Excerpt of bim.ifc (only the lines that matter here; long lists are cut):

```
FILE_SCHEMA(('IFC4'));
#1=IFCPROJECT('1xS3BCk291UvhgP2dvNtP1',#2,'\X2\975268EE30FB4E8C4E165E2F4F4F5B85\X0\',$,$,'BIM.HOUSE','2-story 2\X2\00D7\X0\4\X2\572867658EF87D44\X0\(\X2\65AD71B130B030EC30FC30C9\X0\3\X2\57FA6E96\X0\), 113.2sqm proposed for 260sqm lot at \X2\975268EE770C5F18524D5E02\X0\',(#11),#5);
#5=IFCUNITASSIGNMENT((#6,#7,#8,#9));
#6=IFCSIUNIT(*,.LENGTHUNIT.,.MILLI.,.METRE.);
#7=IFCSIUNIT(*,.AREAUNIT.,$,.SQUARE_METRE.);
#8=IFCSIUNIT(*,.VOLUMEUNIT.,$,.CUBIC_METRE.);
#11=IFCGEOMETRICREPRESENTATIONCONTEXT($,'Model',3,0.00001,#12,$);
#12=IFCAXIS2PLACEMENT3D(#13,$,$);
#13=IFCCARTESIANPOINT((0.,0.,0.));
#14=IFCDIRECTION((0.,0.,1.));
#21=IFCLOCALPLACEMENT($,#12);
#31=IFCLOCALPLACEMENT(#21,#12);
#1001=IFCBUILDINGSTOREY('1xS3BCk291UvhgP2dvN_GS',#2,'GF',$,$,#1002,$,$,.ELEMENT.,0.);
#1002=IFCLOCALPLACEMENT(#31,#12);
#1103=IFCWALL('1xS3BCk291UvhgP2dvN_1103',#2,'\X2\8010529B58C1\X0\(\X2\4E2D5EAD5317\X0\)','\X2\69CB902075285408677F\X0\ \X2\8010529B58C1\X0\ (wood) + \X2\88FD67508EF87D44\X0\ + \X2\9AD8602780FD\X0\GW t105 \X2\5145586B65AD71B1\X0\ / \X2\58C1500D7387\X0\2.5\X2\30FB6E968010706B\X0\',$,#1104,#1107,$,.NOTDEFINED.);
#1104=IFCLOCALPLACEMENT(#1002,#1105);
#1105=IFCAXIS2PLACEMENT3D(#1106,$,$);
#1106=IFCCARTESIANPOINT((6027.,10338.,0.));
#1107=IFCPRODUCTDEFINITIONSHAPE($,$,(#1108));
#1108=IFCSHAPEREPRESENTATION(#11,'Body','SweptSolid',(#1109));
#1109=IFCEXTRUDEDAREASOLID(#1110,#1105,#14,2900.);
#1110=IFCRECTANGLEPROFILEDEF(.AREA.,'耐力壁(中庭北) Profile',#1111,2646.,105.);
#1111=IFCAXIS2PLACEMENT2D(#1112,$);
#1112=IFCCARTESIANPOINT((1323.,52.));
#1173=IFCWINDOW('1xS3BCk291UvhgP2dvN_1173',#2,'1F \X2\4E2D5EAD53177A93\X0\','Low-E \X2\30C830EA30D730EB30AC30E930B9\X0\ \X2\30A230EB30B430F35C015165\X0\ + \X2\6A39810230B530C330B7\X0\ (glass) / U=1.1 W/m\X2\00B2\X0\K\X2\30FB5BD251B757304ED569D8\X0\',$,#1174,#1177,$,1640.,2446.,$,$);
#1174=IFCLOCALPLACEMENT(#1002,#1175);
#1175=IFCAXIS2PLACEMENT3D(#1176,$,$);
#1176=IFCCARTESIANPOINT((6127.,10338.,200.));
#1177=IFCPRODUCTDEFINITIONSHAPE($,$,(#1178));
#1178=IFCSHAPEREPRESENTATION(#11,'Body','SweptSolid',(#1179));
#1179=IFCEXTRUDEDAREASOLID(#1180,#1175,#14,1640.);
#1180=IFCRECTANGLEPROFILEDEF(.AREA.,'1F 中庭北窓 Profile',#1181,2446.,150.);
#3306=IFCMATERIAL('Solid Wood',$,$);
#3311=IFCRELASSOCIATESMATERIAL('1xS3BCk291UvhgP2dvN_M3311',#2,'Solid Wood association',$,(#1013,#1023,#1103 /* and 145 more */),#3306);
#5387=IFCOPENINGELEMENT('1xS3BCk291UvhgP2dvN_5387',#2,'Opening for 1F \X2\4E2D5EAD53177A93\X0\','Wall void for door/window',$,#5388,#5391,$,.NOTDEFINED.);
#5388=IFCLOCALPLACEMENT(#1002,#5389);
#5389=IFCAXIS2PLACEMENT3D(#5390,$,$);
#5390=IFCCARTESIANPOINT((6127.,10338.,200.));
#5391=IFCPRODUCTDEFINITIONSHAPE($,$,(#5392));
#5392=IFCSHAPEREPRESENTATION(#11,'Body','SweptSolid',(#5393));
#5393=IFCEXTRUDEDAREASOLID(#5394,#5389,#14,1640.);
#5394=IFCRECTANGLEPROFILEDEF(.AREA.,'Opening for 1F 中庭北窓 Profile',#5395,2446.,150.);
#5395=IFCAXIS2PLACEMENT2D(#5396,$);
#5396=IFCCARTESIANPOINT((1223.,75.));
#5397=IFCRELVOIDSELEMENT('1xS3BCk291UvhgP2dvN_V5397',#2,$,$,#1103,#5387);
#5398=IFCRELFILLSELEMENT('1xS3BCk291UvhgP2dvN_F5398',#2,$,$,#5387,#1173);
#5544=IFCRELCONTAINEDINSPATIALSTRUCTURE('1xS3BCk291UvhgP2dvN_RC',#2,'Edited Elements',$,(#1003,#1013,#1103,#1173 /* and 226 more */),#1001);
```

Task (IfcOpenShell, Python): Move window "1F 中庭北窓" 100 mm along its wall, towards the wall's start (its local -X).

```python
import ifcopenshell
import ifcopenshell.api.geometry
import ifcopenshell.util.placement

model = ifcopenshell.open("bim.ifc")

window = model.by_guid("1xS3BCk291UvhgP2dvN_1173")
opening = window.FillsVoids[0].RelatingOpeningElement
wall = opening.VoidsElements[0].RelatingBuildingElement

wall_matrix = ifcopenshell.util.placement.get_local_placement(wall.ObjectPlacement)
shift = wall_matrix[:3, 0] * -100.0
before = ifcopenshell.util.placement.get_local_placement(window.ObjectPlacement)[:3, 3].copy()

# The window is not placed relative to its opening, so move both.
for product in (opening, window):
    matrix = ifcopenshell.util.placement.get_local_placement(product.ObjectPlacement)
    matrix[:3, 3] += shift
    ifcopenshell.api.geometry.edit_object_placement(model, product=product, matrix=matrix, is_si=False)

after = ifcopenshell.util.placement.get_local_placement(window.ObjectPlacement)[:3, 3]
print("window moved by", (after - before).round(3) + 0.0)

model.write("bim_v2.ifc")
```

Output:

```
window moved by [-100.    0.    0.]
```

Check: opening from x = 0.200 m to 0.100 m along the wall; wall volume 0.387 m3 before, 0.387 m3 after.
